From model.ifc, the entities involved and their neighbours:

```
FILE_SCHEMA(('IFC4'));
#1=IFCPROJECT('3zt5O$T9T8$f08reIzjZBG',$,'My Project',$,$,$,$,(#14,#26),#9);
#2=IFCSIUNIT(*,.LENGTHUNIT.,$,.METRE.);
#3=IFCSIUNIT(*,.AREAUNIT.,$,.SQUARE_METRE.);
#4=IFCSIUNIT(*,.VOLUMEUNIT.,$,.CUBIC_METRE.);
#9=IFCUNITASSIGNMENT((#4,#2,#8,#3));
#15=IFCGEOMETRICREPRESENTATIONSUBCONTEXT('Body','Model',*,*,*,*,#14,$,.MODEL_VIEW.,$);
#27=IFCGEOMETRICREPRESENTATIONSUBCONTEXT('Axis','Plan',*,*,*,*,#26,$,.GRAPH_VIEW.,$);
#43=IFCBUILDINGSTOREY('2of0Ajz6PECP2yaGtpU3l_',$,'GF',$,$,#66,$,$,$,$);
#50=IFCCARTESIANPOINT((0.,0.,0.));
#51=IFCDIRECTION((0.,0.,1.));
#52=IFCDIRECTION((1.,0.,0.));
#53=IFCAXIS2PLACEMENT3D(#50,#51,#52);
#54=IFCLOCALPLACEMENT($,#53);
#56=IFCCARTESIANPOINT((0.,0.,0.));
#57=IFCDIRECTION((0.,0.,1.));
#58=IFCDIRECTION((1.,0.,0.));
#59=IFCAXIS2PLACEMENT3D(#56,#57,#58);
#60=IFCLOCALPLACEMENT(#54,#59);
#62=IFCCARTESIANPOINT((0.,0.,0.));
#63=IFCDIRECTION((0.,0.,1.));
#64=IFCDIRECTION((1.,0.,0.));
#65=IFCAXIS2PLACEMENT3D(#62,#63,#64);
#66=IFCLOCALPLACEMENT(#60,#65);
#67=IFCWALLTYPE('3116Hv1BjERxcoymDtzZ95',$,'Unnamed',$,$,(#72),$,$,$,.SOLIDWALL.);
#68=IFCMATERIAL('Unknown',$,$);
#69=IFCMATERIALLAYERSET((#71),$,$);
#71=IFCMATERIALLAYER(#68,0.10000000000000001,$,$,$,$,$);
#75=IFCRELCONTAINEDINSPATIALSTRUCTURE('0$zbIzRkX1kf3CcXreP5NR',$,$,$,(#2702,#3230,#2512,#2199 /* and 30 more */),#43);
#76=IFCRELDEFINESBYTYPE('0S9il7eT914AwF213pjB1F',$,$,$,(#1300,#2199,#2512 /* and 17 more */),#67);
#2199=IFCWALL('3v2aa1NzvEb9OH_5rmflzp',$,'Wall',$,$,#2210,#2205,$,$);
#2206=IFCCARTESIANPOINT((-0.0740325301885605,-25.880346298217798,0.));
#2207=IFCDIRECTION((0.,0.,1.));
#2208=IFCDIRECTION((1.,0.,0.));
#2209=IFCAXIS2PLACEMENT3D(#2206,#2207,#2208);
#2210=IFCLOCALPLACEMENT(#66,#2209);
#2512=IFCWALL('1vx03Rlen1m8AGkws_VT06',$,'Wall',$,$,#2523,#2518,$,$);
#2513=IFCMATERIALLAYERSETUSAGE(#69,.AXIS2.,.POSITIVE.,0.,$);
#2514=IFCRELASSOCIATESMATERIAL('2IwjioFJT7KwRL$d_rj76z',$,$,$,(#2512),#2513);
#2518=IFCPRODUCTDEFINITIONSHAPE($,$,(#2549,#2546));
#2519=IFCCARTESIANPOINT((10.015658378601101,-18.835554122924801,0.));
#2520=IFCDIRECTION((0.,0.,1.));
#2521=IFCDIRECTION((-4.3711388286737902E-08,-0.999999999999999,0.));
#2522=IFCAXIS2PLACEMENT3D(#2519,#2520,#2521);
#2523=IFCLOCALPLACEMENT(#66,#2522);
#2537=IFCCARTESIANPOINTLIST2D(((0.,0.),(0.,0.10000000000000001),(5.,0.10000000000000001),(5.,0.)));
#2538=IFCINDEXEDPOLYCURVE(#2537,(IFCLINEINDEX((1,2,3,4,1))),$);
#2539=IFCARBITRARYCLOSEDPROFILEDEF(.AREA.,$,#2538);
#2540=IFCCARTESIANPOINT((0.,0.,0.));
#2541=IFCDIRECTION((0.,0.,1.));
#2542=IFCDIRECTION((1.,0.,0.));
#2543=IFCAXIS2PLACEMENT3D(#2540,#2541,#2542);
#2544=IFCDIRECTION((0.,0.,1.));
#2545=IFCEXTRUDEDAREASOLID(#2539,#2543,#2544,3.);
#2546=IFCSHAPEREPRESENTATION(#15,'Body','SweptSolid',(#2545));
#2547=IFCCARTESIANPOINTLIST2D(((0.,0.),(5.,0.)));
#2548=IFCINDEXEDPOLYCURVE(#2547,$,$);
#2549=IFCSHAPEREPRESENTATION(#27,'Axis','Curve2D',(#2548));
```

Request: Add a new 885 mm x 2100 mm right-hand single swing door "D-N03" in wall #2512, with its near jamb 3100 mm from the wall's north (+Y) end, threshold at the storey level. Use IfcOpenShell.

```python
import numpy as np
import ifcopenshell
import ifcopenshell.api.feature
import ifcopenshell.api.geometry
import ifcopenshell.api.root
import ifcopenshell.api.spatial
import ifcopenshell.geom
import ifcopenshell.util.element
import ifcopenshell.util.placement
import ifcopenshell.util.representation
import ifcopenshell.util.shape
import ifcopenshell.util.unit

model = ifcopenshell.open("model.ifc")
unit_scale = ifcopenshell.util.unit.calculate_unit_scale(model)
settings = ifcopenshell.geom.settings()


def volume(element):
    """Net volume in cubic metres, openings subtracted."""
    shape = ifcopenshell.geom.create_shape(settings, element)
    return ifcopenshell.util.shape.get_volume(shape.geometry)


wall = model.by_id(2512)
storey = ifcopenshell.util.element.get_container(wall, ifc_class="IfcBuildingStorey")
context = ifcopenshell.util.representation.get_context(model, "Model", "Body", "MODEL_VIEW")
before = volume(wall)

width, height, from_end, sill = 0.885, 2.1, 3.1, 0.0  # metres

# The wall runs along its own X axis, and the end named is its -X end.
wall_shape = ifcopenshell.geom.create_shape(settings, wall)
x, y, z = ifcopenshell.util.shape.get_vertices(wall_shape.geometry).T
start = x.min() + from_end
face, thickness = float(y.min()), float(y.max() - y.min())
wall_matrix = ifcopenshell.util.placement.get_local_placement(wall.ObjectPlacement)
level = ifcopenshell.util.placement.get_local_placement(storey.ObjectPlacement)[2, 3]


def in_wall(x, y):
    """Placement at x, y metres in the wall's axes, at sill height."""
    matrix = wall_matrix.copy()
    matrix[:, 3] = wall_matrix @ np.array([x / unit_scale, y / unit_scale, 0.0, 1.0])
    matrix[2, 3] = level + sill / unit_scale
    return matrix


# Opening: a box that overshoots both wall faces by 50 mm.
opening = ifcopenshell.api.root.create_entity(model, ifc_class="IfcOpeningElement", predefined_type="OPENING")
box = ifcopenshell.api.geometry.add_wall_representation(
    model, context=context, length=width, height=height, thickness=thickness + 0.1
)
ifcopenshell.api.geometry.assign_representation(model, product=opening, representation=box)
ifcopenshell.api.geometry.edit_object_placement(model, product=opening, matrix=in_wall(start, face - 0.05), is_si=False)
ifcopenshell.api.feature.add_feature(model, feature=opening, element=wall)

door = ifcopenshell.api.root.create_entity(model, ifc_class="IfcDoor", name="D-N03", predefined_type="DOOR")
door.OverallWidth, door.OverallHeight = width / unit_scale, height / unit_scale
door.OperationType = "SINGLE_SWING_RIGHT"
body = ifcopenshell.api.geometry.add_door_representation(
    model,
    context=context,
    overall_width=door.OverallWidth,
    overall_height=door.OverallHeight,
    operation_type="SINGLE_SWING_RIGHT",
    lining_properties={"LiningDepth": thickness / unit_scale, "ThresholdDepth": thickness / unit_scale},
)
ifcopenshell.api.geometry.assign_representation(model, product=door, representation=body)
ifcopenshell.api.spatial.assign_container(model, products=[door], relating_structure=storey)
ifcopenshell.api.feature.add_filling(model, opening=opening, element=door)

# The lining spans the wall, so the door starts at the wall face.
ifcopenshell.api.geometry.edit_object_placement(model, product=door, matrix=in_wall(start, face), is_si=False)

after = volume(wall)

print(f"wall volume {before:.3f} -> {after:.3f} m3")

model.write("model-out.ifc")
```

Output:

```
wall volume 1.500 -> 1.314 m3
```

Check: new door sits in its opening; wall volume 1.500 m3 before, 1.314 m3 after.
